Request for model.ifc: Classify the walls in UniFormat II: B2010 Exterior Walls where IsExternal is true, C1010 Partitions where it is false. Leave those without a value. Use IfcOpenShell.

First a look at what the model holds.

```python
import ifcopenshell
import ifcopenshell.util.element

model = ifcopenshell.open("model.ifc")
print(model.schema)
print("classifications:", [c.Name for c in model.by_type("IfcClassification")])
values = [ifcopenshell.util.element.get_pset(e, "Pset_WallCommon", "IsExternal") for e in model.by_type("IfcWall")]
for value in (True, False, None):
    print("IsExternal", value, values.count(value))
```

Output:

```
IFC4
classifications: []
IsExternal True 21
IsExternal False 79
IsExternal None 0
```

```python
import ifcopenshell
import ifcopenshell.api.classification
import ifcopenshell.util.element

model = ifcopenshell.open("model.ifc")

system = ifcopenshell.api.classification.add_classification(model, classification="UniFormat II")

walls = model.by_type("IfcWall")
external = {e: ifcopenshell.util.element.get_pset(e, "Pset_WallCommon", "IsExternal") for e in walls}
for flag, code, name in ((True, "B2010", "Exterior Walls"), (False, "C1010", "Partitions")):
    products = [e for e in walls if external[e] is flag]
    ifcopenshell.api.classification.add_reference(
        model, products=products, classification=system, identification=code, name=name
    )
    print(code, len(products))

model.write("model_v2.ifc")
```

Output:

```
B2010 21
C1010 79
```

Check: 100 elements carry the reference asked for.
